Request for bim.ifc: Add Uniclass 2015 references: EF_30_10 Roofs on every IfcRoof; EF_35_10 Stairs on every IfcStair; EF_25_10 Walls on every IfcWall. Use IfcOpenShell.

First a look at what the model holds.

```python
import ifcopenshell

model = ifcopenshell.open("bim.ifc")
print(model.schema)
print("classifications:", [c.Name for c in model.by_type("IfcClassification")])
for ifc_class in ("IfcDoor", "IfcRoof", "IfcStair", "IfcWall", "IfcWindow"):
    print(ifc_class, len(model.by_type(ifc_class)))
```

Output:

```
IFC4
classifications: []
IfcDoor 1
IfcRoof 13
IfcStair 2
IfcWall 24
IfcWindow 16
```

```python
import ifcopenshell
import ifcopenshell.api.classification

model = ifcopenshell.open("bim.ifc")

system = ifcopenshell.api.classification.add_classification(model, classification="Uniclass 2015")

codes = {
    "IfcRoof": ("EF_30_10", "Roofs"),
    "IfcStair": ("EF_35_10", "Stairs"),
    "IfcWall": ("EF_25_10", "Walls"),
}
for ifc_class, (code, name) in codes.items():
    products = model.by_type(ifc_class)
    ifcopenshell.api.classification.add_reference(
        model, products=products, classification=system, identification=code, name=name
    )
    print(code, len(products))

model.write("bim_v2.ifc")
```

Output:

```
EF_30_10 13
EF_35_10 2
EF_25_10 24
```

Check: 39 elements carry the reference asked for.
